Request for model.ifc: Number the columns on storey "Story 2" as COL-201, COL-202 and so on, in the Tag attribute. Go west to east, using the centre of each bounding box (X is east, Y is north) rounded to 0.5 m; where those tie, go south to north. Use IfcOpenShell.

First a look at what the model holds.

```python
import ifcopenshell
import ifcopenshell.util.element
import ifcopenshell.util.placement

model = ifcopenshell.open("model.ifc")
print(model.schema)
storey = next(s for s in model.by_type("IfcBuildingStorey") if s.Name == "Story 2")
columns = [e for e in ifcopenshell.util.element.get_decomposition(storey) if e.is_a("IfcColumn")]
for e in sorted(columns, key=lambda e: e.id()):
    origin = ifcopenshell.util.placement.get_local_placement(e.ObjectPlacement)[:3, 3]
    print(e.id(), e.Tag, e.Name, origin.round(2) + 0.0, sep=" | ")
```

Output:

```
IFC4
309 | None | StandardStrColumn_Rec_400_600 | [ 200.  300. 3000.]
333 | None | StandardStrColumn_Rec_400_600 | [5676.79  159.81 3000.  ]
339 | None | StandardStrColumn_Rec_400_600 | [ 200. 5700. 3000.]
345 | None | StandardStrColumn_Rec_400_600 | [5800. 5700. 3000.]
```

```python
import ifcopenshell
import ifcopenshell.geom
import ifcopenshell.util.element
import ifcopenshell.util.shape

model = ifcopenshell.open("model.ifc")
settings = ifcopenshell.geom.settings()
settings.set("use-world-coords", True)


def centre(element):
    shape = ifcopenshell.geom.create_shape(settings, element)
    return ifcopenshell.util.shape.get_bbox_centroid(shape.geometry)


storey = next(s for s in model.by_type("IfcBuildingStorey") if s.Name == "Story 2")
columns = [e for e in ifcopenshell.util.element.get_decomposition(storey) if e.is_a("IfcColumn")]

# Insertion points can sit at a corner or the storey origin, so sort by the geometry (in metres).
centres = {e: centre(e) for e in columns}
columns.sort(key=lambda e: (round(centres[e][0] / 0.5), centres[e][1]))

for i, e in enumerate(columns, start=1):
    number = f"COL-2{i:02d}"
    e.Tag = number
    print(e.id(), number)

model.write("model_edited.ifc")
```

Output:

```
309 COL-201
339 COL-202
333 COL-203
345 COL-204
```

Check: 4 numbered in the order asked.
